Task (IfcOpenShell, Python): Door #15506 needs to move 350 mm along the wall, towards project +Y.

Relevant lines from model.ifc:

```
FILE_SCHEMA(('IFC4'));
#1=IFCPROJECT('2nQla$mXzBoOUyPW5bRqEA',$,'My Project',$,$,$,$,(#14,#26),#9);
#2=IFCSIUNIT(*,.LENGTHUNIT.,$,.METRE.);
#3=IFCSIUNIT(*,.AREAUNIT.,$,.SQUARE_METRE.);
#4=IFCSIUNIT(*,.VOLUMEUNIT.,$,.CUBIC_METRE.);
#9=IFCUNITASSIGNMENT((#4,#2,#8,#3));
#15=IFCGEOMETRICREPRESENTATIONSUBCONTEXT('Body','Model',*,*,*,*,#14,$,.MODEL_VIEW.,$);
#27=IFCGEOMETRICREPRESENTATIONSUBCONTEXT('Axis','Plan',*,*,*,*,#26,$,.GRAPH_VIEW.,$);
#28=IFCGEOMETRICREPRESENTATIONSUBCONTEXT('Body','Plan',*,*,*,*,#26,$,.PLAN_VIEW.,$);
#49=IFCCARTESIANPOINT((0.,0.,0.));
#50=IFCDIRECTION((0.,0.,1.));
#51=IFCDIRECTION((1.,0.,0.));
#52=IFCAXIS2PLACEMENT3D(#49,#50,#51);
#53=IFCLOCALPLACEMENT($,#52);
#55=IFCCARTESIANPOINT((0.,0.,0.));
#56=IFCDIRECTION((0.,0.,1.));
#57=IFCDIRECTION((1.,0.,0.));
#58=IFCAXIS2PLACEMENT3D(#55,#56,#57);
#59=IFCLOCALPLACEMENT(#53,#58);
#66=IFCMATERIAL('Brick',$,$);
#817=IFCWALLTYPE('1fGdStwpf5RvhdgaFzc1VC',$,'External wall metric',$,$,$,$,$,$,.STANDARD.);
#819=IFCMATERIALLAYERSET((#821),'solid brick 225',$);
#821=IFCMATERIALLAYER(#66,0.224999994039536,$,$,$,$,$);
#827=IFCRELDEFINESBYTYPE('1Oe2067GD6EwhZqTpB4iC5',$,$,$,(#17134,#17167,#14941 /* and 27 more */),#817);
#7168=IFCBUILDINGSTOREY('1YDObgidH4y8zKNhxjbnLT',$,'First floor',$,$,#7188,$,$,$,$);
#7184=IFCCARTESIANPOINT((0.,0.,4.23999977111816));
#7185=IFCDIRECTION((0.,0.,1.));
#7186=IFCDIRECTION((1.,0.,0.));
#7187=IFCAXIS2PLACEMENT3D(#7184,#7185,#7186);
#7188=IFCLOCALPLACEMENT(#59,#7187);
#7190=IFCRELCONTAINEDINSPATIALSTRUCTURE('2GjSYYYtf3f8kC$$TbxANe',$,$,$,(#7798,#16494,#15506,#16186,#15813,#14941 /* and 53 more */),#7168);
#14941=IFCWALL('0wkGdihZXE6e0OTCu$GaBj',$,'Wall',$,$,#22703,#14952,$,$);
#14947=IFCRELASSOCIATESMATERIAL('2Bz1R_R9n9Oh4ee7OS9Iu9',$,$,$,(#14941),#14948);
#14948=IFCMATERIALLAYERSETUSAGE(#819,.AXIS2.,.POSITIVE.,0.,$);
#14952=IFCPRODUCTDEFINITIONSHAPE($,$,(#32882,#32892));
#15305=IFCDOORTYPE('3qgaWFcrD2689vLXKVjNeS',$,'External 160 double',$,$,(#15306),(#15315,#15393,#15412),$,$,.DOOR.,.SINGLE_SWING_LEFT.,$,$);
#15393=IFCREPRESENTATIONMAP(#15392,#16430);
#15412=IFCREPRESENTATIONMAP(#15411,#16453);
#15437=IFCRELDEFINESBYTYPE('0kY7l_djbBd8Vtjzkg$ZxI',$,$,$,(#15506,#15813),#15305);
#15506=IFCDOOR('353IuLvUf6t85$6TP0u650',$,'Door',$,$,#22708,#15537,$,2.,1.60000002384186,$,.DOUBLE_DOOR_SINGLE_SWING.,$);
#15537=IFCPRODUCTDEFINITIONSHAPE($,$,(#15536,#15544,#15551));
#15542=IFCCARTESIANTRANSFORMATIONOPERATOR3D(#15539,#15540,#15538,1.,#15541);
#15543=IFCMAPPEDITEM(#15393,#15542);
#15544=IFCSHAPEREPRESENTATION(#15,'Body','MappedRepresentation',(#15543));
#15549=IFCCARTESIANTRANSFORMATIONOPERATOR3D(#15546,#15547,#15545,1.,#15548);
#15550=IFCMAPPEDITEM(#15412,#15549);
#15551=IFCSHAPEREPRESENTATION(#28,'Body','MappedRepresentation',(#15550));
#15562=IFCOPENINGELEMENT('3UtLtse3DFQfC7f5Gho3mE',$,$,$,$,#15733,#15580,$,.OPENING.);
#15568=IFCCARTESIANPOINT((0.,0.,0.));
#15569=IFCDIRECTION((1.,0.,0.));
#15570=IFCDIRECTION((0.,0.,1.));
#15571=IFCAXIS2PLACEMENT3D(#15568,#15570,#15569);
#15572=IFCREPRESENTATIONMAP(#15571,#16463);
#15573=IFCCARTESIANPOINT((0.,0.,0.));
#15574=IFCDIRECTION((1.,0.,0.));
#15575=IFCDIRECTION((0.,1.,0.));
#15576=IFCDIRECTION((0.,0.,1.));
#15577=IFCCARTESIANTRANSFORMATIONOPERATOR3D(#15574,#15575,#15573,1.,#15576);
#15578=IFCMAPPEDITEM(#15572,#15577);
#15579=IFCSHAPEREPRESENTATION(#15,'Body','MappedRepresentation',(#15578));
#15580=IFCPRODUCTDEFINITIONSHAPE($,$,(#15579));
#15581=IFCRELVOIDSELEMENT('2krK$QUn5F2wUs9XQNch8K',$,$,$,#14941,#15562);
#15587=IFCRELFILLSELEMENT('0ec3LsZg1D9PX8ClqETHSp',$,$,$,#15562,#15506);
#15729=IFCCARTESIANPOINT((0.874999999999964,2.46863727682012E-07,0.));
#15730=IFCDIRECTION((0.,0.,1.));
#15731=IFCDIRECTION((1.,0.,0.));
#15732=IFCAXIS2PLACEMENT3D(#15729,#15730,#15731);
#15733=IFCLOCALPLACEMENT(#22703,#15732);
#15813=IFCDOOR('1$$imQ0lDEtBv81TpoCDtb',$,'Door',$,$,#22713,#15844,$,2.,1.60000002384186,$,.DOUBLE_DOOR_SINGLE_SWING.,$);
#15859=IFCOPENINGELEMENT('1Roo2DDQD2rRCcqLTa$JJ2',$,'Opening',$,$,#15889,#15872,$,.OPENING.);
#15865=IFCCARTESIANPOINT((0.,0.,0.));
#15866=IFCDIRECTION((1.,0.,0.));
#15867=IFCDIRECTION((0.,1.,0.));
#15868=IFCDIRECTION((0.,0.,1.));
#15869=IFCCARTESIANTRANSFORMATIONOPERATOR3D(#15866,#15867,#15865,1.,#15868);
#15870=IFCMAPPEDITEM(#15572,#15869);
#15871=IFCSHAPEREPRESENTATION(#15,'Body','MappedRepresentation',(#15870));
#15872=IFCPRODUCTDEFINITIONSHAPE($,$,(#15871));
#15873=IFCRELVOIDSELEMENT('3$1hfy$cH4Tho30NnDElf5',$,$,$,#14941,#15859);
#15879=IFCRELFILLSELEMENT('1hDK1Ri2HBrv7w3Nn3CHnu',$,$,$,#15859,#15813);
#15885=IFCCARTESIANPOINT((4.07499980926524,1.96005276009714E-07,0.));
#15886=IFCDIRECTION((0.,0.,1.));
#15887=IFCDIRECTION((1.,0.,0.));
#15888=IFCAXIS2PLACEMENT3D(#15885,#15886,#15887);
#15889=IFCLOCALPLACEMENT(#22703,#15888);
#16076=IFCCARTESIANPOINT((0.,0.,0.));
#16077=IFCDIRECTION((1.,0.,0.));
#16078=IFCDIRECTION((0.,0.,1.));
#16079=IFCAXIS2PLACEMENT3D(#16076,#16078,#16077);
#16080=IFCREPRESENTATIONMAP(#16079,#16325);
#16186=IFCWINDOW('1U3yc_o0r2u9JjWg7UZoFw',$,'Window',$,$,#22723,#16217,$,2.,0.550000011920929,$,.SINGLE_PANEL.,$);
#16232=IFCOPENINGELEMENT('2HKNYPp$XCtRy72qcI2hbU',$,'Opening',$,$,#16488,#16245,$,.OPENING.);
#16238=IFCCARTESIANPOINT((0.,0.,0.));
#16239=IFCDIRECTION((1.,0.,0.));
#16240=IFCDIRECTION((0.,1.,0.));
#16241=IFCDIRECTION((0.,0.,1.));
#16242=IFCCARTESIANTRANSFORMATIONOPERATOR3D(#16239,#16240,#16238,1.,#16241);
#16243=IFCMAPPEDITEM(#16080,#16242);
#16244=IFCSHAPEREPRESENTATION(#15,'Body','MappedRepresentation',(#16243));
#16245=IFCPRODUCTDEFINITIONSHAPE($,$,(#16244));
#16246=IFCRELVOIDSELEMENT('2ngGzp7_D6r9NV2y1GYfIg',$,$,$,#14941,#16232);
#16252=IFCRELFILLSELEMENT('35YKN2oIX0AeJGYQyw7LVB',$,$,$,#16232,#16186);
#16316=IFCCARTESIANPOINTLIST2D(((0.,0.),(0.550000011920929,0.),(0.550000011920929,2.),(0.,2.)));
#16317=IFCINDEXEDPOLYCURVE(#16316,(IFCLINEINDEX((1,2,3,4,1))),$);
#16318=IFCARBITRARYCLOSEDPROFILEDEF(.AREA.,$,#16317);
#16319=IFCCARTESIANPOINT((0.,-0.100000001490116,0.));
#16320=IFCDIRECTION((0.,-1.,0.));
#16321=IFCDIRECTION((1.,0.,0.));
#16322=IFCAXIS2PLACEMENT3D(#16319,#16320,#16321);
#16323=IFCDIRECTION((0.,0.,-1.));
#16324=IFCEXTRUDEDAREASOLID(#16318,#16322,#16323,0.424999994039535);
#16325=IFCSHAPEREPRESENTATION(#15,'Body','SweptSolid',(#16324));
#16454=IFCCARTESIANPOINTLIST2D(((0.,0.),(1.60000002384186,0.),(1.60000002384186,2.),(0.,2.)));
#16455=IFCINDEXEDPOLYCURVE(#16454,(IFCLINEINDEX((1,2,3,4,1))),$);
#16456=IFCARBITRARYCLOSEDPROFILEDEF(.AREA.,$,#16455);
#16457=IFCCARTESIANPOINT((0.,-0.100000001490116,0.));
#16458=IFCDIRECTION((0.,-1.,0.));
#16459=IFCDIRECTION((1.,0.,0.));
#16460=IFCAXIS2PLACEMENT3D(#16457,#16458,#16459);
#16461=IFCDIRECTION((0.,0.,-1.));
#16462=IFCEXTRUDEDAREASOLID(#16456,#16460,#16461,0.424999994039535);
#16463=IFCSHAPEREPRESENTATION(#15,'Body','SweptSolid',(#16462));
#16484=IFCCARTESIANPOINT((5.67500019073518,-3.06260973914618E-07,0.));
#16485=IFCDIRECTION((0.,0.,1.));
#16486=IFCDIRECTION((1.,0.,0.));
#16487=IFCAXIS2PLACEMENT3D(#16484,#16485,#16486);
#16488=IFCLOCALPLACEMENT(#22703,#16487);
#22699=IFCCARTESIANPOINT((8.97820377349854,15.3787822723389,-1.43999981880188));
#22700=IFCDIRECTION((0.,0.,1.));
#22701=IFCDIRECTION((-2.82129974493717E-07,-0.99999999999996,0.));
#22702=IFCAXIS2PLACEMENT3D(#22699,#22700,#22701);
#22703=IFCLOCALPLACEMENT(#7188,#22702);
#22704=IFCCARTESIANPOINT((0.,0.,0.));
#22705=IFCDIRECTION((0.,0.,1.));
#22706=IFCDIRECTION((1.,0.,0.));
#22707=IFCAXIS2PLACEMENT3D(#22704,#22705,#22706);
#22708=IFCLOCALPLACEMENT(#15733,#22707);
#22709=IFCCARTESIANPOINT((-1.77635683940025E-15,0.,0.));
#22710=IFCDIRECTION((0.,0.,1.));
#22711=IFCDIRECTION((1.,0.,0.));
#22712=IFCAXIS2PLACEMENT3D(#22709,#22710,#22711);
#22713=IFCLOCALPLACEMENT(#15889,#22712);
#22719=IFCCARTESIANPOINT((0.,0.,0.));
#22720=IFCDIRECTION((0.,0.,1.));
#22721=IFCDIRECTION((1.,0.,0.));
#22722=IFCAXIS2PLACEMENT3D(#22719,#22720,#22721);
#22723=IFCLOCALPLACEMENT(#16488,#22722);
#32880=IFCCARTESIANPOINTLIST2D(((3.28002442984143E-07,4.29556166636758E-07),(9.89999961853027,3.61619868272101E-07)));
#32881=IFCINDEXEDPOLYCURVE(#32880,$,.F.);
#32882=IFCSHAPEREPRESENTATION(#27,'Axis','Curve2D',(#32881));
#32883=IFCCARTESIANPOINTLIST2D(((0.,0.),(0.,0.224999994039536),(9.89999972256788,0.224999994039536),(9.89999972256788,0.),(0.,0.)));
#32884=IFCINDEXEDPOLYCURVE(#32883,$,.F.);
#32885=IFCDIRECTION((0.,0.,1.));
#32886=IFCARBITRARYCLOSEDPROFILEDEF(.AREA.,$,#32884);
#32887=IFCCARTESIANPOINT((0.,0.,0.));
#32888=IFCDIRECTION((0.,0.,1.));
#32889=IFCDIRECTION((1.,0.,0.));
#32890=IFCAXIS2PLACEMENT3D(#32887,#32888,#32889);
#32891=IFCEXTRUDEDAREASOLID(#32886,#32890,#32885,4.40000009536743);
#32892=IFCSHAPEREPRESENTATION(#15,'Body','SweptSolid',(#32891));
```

```python
import ifcopenshell
import ifcopenshell.api.geometry
import ifcopenshell.util.placement
import ifcopenshell.util.unit

model = ifcopenshell.open("model.ifc")
unit_scale = ifcopenshell.util.unit.calculate_unit_scale(model)

door = model.by_guid("353IuLvUf6t85$6TP0u650")
opening = door.FillsVoids[0].RelatingOpeningElement
wall = opening.VoidsElements[0].RelatingBuildingElement

wall_matrix = ifcopenshell.util.placement.get_local_placement(wall.ObjectPlacement)
shift = wall_matrix[:3, 0] * -0.35 / unit_scale
before = ifcopenshell.util.placement.get_local_placement(door.ObjectPlacement)[:3, 3].copy()

# The door is placed relative to its opening, so it follows when the opening moves.
matrix = ifcopenshell.util.placement.get_local_placement(opening.ObjectPlacement)
matrix[:3, 3] += shift
ifcopenshell.api.geometry.edit_object_placement(
    model, product=opening, matrix=matrix, is_si=False, should_transform_children=True
)

after = ifcopenshell.util.placement.get_local_placement(door.ObjectPlacement)[:3, 3]
print("door moved by", (after - before).round(3) + 0.0)

model.write("model_rev.ifc")
```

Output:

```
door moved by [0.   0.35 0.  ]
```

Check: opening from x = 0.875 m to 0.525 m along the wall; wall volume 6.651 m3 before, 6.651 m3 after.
